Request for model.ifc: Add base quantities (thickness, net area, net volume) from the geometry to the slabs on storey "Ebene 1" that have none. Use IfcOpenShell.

First a look at what the model holds.

```python
import ifcopenshell
import ifcopenshell.util.element
import ifcopenshell.util.unit

model = ifcopenshell.open("model.ifc")
print(model.schema)
for unit_type in ("LENGTHUNIT", "AREAUNIT", "VOLUMEUNIT"):
    print(unit_type, ifcopenshell.util.unit.calculate_unit_scale(model, unit_type))
storey = next(s for s in model.by_type("IfcBuildingStorey") if s.Name == "Ebene 1")
slabs = [e for e in ifcopenshell.util.element.get_decomposition(storey) if e.is_a("IfcSlab")]
for e in sorted(slabs, key=lambda e: e.id()):
    print(e.id(), e.is_a(), e.Name, list(ifcopenshell.util.element.get_psets(e, qtos_only=True)), sep=" | ")
```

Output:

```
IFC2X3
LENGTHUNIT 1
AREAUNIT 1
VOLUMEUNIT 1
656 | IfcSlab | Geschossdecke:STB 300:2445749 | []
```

```python
import ifcopenshell
import ifcopenshell.api.pset
import ifcopenshell.geom
import ifcopenshell.util.element
import ifcopenshell.util.shape
import ifcopenshell.util.unit

model = ifcopenshell.open("model.ifc")
unit_scale = ifcopenshell.util.unit.calculate_unit_scale(model)
area_scale = ifcopenshell.util.unit.calculate_unit_scale(model, "AREAUNIT")
volume_scale = ifcopenshell.util.unit.calculate_unit_scale(model, "VOLUMEUNIT")
settings = ifcopenshell.geom.settings()

storey = next(s for s in model.by_type("IfcBuildingStorey") if s.Name == "Ebene 1")
slabs = [e for e in ifcopenshell.util.element.get_decomposition(storey) if e.is_a("IfcSlab")]

for e in sorted(slabs, key=lambda e: e.id()):
    if ifcopenshell.util.element.get_psets(e, qtos_only=True, should_inherit=False):
        continue
    # Geometry comes back in metres, in the element's own axes.
    shape = ifcopenshell.geom.create_shape(settings, e)
    values = {
        "Width": ifcopenshell.util.shape.get_z(shape.geometry) / unit_scale,
        "NetArea": ifcopenshell.util.shape.get_footprint_area(shape.geometry) / area_scale,
        "NetVolume": ifcopenshell.util.shape.get_volume(shape.geometry) / volume_scale,
    }
    qto = ifcopenshell.api.pset.add_qto(model, product=e, name="BaseQuantities")
    ifcopenshell.api.pset.edit_qto(model, qto=qto, properties=values)
    print(e.id(), {k: round(v, 3) for k, v in values.items()})

model.write("model-out.ifc")
```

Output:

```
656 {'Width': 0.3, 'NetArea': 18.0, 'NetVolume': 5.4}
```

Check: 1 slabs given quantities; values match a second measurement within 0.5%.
